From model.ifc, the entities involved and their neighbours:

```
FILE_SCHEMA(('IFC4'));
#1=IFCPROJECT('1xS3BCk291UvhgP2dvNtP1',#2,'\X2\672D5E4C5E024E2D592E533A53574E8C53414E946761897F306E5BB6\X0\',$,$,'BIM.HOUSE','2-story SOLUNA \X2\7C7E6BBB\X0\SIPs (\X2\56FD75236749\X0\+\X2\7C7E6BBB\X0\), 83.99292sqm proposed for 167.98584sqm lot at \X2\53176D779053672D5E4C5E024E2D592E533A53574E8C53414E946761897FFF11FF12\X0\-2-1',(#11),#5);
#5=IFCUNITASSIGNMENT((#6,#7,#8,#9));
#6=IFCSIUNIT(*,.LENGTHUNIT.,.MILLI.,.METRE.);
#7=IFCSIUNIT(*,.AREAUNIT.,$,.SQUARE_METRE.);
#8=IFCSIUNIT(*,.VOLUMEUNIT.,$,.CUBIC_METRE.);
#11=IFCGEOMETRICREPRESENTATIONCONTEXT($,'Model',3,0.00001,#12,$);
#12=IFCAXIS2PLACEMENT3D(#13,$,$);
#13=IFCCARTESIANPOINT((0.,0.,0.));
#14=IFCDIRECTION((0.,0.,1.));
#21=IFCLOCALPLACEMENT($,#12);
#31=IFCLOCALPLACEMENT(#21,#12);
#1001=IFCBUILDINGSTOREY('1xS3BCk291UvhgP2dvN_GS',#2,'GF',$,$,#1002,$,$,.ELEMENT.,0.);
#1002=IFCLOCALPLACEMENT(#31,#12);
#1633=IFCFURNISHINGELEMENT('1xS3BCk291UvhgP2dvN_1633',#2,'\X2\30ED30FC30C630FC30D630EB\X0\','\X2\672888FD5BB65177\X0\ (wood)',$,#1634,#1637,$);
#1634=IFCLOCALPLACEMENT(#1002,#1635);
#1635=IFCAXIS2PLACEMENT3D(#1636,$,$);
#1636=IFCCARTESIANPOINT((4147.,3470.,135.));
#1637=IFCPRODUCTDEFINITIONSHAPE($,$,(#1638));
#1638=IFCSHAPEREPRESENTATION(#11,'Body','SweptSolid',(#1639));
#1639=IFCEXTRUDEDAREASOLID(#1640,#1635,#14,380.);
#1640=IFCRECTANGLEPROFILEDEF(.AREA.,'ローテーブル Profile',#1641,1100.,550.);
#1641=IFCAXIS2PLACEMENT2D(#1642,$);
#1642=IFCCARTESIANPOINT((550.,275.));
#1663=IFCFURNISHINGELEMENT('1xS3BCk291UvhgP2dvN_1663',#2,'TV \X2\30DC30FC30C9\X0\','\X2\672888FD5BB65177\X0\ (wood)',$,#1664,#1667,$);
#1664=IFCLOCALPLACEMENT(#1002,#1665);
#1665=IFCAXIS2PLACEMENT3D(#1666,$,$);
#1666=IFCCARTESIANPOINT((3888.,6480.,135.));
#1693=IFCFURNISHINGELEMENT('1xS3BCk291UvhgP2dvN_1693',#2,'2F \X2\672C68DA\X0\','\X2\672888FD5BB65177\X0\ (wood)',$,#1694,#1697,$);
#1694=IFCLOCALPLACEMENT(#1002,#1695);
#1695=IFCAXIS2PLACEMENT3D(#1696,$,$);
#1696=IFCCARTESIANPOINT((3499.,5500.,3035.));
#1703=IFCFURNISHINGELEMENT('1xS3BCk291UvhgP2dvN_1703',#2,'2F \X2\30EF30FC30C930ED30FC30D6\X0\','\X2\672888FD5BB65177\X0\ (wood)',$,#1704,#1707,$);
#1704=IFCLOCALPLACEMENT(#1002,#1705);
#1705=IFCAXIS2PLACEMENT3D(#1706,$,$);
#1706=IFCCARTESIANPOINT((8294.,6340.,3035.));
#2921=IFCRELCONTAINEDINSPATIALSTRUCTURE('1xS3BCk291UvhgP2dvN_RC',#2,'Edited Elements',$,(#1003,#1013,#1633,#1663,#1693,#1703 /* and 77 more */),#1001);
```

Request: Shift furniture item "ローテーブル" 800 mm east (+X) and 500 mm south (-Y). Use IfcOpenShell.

```python
import ifcopenshell
import ifcopenshell.api.geometry
import ifcopenshell.util.placement

model = ifcopenshell.open("model.ifc")

item = model.by_guid("1xS3BCk291UvhgP2dvN_1633")
matrix = ifcopenshell.util.placement.get_local_placement(item.ObjectPlacement)
matrix[0, 3] += 800.0
matrix[1, 3] -= 500.0
ifcopenshell.api.geometry.edit_object_placement(model, product=item, matrix=matrix, is_si=False)

print(ifcopenshell.util.placement.get_local_placement(item.ObjectPlacement).round(3) + 0.0)

model.write("model_v2.ifc")
```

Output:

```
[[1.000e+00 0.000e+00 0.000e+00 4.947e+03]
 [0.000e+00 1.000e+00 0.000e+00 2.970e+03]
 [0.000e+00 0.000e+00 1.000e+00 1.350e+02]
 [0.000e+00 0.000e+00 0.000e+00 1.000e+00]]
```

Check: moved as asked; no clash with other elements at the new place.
